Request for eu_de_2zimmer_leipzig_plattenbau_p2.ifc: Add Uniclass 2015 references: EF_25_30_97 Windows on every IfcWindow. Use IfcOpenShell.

First a look at what the model holds.

```python
import ifcopenshell

model = ifcopenshell.open("eu_de_2zimmer_leipzig_plattenbau_p2.ifc")
print(model.schema)
print("classifications:", [c.Name for c in model.by_type("IfcClassification")])
for ifc_class in ("IfcDoor", "IfcRoof", "IfcStair", "IfcWall", "IfcWindow"):
    print(ifc_class, len(model.by_type(ifc_class)))
```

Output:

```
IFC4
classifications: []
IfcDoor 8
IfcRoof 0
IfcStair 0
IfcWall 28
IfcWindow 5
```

```python
import ifcopenshell
import ifcopenshell.api.classification

model = ifcopenshell.open("eu_de_2zimmer_leipzig_plattenbau_p2.ifc")

system = ifcopenshell.api.classification.add_classification(model, classification="Uniclass 2015")

codes = {
    "IfcWindow": ("EF_25_30_97", "Windows"),
}
for ifc_class, (code, name) in codes.items():
    products = model.by_type(ifc_class)
    ifcopenshell.api.classification.add_reference(
        model, products=products, classification=system, identification=code, name=name
    )
    print(code, len(products))

model.write("eu_de_2zimmer_leipzig_plattenbau_p2_edited.ifc")
```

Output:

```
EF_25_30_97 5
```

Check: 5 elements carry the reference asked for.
